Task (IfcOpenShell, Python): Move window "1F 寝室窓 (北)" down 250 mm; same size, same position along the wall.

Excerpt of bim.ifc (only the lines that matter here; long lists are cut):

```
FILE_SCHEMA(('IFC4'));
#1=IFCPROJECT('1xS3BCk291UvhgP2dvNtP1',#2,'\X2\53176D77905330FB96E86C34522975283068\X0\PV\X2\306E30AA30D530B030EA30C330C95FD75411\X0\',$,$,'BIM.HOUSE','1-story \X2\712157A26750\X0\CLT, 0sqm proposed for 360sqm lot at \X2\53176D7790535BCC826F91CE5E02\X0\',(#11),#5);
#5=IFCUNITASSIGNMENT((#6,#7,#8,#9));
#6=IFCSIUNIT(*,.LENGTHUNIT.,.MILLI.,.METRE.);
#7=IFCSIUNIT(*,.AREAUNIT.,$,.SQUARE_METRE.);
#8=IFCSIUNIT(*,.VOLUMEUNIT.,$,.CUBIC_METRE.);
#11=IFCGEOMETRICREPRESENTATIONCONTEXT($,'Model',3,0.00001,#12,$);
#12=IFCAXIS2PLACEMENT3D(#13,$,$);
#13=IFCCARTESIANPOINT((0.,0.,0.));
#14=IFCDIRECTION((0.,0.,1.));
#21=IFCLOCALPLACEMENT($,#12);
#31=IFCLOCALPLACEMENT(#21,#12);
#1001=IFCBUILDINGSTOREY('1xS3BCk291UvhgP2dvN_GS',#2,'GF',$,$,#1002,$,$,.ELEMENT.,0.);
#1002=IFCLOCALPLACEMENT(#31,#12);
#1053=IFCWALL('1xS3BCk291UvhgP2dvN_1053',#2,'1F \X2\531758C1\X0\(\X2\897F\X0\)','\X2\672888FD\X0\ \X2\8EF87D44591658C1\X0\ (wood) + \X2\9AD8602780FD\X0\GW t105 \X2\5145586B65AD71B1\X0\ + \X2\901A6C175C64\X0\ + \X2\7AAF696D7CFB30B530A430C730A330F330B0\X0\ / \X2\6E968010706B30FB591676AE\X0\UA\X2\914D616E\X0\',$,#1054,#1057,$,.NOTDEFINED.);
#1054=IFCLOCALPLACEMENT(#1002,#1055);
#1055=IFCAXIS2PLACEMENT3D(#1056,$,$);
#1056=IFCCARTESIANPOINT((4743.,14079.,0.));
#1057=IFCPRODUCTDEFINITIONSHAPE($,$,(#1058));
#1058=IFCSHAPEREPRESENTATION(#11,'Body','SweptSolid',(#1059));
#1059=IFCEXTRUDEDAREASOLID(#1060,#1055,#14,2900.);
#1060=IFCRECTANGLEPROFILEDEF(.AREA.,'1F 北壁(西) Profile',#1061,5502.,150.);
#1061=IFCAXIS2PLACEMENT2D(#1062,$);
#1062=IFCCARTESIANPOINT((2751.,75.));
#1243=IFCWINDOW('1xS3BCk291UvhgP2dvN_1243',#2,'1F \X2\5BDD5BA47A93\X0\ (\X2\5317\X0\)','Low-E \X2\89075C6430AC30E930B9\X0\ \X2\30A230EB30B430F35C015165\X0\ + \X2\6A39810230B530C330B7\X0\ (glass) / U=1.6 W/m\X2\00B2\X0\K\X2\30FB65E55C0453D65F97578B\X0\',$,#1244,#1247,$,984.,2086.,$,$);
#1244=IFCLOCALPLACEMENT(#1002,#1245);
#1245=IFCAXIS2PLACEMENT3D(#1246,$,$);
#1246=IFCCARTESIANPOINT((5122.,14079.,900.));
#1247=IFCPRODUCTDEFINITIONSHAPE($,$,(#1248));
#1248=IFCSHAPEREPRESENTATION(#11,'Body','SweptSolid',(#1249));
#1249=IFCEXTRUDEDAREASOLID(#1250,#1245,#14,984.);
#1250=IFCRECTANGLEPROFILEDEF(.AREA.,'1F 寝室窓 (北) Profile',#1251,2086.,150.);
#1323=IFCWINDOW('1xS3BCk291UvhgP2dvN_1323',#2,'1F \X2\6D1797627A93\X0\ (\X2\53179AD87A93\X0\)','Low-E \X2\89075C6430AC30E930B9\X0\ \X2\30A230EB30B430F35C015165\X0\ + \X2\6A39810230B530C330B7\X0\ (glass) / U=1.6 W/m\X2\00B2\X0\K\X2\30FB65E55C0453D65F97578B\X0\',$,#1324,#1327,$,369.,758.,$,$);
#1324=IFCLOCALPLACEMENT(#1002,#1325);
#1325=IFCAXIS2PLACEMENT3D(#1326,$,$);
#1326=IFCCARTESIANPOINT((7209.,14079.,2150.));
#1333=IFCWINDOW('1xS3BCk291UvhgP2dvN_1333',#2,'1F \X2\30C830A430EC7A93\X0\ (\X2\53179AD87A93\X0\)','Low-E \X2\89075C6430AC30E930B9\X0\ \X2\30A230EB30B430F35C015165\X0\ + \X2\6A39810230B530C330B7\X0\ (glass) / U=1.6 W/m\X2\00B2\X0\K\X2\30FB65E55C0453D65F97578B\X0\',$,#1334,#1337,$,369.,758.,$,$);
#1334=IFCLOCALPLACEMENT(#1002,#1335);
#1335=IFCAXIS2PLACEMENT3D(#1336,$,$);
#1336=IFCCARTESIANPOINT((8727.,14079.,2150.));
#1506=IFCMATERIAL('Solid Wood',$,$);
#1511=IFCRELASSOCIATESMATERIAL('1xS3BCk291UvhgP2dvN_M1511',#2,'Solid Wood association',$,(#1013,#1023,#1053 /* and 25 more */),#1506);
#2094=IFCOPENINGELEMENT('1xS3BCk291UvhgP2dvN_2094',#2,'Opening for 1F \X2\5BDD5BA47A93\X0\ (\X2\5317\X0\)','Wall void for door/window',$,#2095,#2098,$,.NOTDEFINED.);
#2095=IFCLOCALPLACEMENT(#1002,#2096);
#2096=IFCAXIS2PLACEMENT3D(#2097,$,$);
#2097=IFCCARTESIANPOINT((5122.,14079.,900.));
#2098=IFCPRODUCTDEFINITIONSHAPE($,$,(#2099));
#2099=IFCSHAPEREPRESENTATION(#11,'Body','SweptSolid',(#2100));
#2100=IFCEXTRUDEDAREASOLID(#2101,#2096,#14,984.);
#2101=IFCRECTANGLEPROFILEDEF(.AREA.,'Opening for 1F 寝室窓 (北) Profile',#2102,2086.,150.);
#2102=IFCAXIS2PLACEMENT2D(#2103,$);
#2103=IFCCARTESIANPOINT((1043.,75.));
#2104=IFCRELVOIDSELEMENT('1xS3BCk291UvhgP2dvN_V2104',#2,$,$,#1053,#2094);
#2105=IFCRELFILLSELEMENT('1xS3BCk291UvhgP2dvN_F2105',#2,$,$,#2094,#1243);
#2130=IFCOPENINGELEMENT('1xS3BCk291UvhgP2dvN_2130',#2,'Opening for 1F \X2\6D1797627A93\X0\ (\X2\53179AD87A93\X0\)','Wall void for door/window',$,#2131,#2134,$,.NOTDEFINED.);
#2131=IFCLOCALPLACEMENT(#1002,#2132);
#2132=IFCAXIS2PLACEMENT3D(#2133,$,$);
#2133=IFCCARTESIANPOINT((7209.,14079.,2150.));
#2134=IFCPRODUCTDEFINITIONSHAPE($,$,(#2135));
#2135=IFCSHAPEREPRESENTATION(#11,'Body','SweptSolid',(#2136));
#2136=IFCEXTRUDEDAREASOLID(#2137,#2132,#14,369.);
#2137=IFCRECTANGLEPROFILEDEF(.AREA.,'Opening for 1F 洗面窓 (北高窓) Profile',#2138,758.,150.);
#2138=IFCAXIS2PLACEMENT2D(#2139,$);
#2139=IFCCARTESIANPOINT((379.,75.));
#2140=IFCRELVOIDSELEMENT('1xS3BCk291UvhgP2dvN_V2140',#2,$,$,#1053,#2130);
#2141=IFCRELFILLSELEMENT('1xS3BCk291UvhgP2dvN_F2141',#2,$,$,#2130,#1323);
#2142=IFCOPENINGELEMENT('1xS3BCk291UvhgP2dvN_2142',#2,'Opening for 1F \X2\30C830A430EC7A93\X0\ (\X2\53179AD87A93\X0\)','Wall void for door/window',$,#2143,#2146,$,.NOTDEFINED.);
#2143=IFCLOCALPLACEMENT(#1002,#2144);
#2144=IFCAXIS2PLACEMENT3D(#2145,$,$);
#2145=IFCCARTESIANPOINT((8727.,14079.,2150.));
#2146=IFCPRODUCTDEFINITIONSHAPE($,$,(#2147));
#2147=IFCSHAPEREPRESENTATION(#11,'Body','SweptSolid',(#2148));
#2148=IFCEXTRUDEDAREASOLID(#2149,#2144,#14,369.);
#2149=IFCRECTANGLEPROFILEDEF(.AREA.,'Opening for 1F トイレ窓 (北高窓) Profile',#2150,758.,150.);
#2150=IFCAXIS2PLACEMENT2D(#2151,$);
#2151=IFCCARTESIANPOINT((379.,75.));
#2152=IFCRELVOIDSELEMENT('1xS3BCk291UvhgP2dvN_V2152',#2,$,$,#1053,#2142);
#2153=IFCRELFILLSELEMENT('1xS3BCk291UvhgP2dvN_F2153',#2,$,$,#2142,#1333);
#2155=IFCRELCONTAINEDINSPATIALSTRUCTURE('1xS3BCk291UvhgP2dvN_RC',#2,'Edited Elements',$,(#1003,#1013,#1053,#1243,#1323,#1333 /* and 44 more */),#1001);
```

```python
import numpy as np
import ifcopenshell
import ifcopenshell.api.geometry
import ifcopenshell.util.placement
import ifcopenshell.util.unit

model = ifcopenshell.open("bim.ifc")
unit_scale = ifcopenshell.util.unit.calculate_unit_scale(model)

window = model.by_guid("1xS3BCk291UvhgP2dvN_1243")
opening = window.FillsVoids[0].RelatingOpeningElement
dz = -250.0

shift = np.array([0.0, 0.0, dz])
# The window is not placed relative to its opening, so move both.
for product in (opening, window):
    matrix = ifcopenshell.util.placement.get_local_placement(product.ObjectPlacement)
    matrix[:3, 3] += shift
    ifcopenshell.api.geometry.edit_object_placement(model, product=product, matrix=matrix, is_si=False)

print(f"moved by {dz * unit_scale:+.3f} m")

model.write("bim_updated.ifc")
```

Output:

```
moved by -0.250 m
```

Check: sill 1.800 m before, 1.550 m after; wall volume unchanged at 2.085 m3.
